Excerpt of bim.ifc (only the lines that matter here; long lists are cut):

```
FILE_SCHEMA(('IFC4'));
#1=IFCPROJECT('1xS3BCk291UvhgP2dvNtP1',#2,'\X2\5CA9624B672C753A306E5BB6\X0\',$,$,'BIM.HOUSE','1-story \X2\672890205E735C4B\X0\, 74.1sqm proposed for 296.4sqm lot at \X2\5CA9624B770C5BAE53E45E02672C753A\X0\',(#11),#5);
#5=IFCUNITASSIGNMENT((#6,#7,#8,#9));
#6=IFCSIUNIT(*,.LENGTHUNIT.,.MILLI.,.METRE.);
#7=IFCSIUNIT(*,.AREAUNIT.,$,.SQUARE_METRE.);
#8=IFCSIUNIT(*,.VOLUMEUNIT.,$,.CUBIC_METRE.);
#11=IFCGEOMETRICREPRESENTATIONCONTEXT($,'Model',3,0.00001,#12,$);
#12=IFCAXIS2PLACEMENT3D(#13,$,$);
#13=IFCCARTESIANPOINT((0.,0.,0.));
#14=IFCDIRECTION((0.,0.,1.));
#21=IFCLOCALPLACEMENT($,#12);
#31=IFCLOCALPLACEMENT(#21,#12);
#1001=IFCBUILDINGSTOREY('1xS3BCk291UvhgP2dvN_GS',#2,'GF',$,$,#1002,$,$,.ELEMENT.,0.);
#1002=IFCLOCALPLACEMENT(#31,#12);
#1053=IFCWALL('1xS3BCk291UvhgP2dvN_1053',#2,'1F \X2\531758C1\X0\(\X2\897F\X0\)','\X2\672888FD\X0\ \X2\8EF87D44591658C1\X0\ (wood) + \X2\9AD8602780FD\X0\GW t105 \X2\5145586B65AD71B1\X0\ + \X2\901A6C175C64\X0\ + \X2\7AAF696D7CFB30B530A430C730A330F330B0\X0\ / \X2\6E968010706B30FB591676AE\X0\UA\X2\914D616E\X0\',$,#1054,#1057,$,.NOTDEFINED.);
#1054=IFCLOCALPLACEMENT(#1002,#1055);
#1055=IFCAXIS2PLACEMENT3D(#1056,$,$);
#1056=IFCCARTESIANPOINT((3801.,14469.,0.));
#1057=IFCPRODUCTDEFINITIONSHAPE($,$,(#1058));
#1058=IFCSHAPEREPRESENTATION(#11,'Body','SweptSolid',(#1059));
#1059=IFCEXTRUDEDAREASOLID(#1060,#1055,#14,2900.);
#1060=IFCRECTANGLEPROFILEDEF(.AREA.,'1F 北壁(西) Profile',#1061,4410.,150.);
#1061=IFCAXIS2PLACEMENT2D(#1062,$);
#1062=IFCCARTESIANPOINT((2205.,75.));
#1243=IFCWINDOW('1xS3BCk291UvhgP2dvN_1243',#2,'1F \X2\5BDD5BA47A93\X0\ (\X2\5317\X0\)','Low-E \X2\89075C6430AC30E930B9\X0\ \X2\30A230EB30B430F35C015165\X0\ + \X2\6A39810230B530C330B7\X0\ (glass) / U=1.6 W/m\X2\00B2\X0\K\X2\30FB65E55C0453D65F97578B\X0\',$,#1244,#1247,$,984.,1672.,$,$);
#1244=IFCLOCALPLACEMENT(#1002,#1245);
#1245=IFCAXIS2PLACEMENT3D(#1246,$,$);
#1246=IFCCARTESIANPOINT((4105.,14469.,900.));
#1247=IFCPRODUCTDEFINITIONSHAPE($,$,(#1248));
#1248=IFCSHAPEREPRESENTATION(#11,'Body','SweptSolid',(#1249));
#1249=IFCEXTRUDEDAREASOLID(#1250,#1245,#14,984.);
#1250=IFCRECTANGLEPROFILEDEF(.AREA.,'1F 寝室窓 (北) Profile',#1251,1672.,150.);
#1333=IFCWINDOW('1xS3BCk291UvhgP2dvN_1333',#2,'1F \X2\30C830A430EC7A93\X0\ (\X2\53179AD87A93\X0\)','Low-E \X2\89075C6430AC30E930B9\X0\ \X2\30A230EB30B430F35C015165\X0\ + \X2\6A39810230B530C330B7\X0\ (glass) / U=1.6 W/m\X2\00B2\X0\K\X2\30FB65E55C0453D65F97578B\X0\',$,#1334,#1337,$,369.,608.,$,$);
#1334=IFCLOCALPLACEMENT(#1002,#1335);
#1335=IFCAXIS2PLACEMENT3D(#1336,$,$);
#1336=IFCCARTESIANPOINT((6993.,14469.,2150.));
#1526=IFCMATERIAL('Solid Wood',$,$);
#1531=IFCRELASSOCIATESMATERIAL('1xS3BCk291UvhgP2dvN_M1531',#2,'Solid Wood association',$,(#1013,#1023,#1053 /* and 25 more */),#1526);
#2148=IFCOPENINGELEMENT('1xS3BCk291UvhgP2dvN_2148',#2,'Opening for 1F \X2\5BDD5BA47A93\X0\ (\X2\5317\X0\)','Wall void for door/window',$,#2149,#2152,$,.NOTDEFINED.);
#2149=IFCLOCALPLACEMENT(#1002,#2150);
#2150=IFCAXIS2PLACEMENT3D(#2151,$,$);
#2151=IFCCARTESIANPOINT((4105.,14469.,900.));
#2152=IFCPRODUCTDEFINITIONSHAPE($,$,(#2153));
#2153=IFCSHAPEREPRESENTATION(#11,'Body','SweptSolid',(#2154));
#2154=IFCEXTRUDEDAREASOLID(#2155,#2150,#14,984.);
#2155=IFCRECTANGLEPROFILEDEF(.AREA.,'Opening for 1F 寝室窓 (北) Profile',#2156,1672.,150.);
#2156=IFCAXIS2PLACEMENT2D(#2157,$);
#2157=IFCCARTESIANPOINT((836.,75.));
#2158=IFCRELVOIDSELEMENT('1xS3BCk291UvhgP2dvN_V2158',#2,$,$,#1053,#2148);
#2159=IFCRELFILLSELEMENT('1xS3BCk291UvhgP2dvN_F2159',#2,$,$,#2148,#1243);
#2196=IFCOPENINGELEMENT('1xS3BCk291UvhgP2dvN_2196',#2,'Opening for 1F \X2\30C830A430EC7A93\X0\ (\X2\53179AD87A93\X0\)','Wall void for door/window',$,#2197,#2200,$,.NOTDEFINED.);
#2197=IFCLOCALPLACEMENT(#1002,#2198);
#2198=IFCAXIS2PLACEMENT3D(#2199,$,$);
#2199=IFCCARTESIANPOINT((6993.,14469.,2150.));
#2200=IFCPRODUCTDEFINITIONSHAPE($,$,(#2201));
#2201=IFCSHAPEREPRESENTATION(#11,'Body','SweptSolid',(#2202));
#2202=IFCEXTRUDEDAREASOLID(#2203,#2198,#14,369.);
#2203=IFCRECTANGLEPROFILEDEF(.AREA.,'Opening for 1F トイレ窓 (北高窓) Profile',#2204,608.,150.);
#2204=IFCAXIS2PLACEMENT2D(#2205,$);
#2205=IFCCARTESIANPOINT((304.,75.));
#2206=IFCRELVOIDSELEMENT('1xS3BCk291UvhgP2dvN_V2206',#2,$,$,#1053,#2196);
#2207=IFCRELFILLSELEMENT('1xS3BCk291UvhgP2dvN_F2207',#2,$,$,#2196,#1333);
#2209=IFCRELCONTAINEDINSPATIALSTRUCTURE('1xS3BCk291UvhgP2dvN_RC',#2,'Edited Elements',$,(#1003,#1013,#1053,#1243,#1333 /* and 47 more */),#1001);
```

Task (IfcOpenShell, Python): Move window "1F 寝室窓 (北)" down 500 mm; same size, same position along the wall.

```python
import numpy as np
import ifcopenshell
import ifcopenshell.api.geometry
import ifcopenshell.util.placement
import ifcopenshell.util.unit

model = ifcopenshell.open("bim.ifc")
unit_scale = ifcopenshell.util.unit.calculate_unit_scale(model)

window = model.by_id(1243)
opening = window.FillsVoids[0].RelatingOpeningElement
dz = -0.5 / unit_scale

shift = np.array([0.0, 0.0, dz])
# The window is not placed relative to its opening, so move both.
for product in (opening, window):
    matrix = ifcopenshell.util.placement.get_local_placement(product.ObjectPlacement)
    matrix[:3, 3] += shift
    ifcopenshell.api.geometry.edit_object_placement(model, product=product, matrix=matrix, is_si=False)

print(f"moved by {dz * unit_scale:+.3f} m")

model.write("bim-out.ifc")
```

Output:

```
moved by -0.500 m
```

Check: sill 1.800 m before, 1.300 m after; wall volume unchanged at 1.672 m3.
